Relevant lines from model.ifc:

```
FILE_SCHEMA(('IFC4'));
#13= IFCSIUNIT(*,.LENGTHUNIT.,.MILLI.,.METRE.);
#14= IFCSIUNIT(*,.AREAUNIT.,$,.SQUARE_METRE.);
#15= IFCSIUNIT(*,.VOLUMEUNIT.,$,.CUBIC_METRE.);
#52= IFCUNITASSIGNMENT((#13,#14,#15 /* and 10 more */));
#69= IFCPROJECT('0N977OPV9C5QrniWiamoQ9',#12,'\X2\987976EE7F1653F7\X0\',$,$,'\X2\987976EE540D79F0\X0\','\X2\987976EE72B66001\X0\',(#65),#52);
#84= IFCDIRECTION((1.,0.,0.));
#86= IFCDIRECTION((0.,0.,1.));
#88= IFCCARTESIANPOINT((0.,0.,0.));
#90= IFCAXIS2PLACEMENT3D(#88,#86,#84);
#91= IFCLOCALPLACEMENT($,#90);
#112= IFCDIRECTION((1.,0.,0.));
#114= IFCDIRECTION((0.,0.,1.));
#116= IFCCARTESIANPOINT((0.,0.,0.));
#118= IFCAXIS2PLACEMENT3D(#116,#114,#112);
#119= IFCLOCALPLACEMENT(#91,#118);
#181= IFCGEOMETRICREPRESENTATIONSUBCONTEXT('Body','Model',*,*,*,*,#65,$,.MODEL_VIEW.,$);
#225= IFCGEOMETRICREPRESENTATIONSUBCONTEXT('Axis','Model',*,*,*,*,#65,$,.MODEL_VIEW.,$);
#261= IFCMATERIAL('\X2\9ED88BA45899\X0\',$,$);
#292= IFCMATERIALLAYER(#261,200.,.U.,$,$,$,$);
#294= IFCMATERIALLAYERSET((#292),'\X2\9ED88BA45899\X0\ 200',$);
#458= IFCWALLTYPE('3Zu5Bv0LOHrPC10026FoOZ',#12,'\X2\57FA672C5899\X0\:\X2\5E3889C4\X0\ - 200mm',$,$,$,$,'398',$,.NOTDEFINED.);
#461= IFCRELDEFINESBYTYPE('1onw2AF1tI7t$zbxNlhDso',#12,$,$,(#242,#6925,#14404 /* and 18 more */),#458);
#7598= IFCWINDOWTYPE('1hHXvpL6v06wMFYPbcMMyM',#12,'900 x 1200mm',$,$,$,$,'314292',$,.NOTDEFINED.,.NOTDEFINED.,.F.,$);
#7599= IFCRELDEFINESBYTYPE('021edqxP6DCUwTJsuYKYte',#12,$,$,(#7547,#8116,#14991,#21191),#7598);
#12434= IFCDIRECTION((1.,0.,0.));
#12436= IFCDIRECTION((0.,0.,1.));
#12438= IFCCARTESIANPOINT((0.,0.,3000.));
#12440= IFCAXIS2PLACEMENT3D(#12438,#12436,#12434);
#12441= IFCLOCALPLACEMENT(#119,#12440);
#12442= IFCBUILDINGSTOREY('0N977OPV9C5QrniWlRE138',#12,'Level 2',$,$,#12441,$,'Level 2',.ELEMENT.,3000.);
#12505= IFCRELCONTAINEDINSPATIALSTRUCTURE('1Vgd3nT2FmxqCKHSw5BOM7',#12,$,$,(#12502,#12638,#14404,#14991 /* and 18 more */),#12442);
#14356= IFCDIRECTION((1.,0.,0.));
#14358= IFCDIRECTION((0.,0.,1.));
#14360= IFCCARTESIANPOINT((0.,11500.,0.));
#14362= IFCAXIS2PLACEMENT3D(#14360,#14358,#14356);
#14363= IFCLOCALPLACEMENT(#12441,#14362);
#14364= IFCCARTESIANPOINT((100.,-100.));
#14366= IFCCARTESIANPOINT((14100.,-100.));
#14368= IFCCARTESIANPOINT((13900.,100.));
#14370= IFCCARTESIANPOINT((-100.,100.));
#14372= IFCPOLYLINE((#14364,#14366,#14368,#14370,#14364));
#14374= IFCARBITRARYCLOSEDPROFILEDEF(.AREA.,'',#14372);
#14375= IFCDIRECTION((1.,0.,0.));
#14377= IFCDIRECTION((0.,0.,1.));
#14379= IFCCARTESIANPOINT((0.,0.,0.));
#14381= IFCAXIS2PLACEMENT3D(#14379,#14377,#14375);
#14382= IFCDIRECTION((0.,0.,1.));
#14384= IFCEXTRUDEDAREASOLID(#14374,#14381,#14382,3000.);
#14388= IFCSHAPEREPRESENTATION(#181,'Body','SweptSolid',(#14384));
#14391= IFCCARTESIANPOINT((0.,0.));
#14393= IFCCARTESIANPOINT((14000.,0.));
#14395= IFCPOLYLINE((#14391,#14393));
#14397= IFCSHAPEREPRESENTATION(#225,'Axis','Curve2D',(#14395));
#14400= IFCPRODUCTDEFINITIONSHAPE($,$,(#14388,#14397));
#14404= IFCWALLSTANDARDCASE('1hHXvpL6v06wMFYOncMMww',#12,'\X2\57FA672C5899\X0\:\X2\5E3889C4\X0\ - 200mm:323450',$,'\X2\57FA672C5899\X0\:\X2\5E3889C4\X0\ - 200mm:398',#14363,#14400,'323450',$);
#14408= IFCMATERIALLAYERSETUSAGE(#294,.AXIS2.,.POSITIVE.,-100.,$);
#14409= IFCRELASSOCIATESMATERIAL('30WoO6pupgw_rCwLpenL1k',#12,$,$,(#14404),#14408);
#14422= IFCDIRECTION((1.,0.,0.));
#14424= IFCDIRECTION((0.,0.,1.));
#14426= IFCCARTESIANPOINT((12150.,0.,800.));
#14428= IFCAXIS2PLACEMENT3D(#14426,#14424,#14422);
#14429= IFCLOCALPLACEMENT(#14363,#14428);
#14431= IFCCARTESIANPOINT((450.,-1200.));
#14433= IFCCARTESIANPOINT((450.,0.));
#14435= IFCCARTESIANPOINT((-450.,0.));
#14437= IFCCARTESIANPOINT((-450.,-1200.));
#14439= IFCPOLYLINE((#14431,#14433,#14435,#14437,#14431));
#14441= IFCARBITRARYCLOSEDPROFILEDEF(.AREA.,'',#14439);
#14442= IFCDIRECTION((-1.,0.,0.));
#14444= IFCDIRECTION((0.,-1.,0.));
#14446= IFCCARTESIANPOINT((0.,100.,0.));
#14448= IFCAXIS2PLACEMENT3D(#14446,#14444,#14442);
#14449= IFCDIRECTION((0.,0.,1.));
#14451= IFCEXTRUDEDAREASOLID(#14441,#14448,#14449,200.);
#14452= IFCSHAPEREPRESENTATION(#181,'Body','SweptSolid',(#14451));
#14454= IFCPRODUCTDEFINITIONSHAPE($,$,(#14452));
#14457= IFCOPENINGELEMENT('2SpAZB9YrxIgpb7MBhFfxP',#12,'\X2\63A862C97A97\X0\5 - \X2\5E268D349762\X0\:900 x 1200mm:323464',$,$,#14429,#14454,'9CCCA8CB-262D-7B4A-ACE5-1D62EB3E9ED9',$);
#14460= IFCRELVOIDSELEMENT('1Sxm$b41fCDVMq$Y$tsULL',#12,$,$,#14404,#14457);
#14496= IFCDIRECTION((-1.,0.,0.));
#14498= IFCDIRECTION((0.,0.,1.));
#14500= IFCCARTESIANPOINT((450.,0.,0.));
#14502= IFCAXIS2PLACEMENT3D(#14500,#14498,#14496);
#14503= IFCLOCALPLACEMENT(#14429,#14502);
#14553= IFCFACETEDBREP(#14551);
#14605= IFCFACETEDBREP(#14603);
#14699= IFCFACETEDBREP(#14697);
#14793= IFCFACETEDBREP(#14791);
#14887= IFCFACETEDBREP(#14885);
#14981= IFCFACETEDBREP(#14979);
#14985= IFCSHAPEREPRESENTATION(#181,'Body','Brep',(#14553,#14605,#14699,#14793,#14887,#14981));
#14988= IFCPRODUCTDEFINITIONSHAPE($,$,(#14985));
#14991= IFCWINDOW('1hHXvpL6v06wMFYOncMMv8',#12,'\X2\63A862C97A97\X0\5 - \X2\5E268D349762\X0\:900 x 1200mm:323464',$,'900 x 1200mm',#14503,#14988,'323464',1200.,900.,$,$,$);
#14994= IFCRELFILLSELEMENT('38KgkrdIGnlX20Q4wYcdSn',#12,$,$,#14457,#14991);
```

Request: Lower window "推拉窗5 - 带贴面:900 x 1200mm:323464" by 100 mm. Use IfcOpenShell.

```python
import numpy as np
import ifcopenshell
import ifcopenshell.api.geometry
import ifcopenshell.util.placement
import ifcopenshell.util.unit

model = ifcopenshell.open("model.ifc")
unit_scale = ifcopenshell.util.unit.calculate_unit_scale(model)

window = model.by_id(14991)
opening = window.FillsVoids[0].RelatingOpeningElement
dz = -100.0

shift = np.array([0.0, 0.0, dz])
# The window is placed relative to its opening, so it follows when the opening moves.
matrix = ifcopenshell.util.placement.get_local_placement(opening.ObjectPlacement)
matrix[:3, 3] += shift
ifcopenshell.api.geometry.edit_object_placement(
    model, product=opening, matrix=matrix, is_si=False, should_transform_children=True
)

print(f"moved by {dz * unit_scale:+.3f} m")

model.write("model_edited.ifc")
```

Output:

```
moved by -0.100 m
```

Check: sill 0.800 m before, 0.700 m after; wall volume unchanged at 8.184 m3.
